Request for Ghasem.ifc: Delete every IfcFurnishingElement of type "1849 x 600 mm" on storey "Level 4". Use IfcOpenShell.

First a look at what the model holds.

```python
import ifcopenshell
import ifcopenshell.util.element

model = ifcopenshell.open("Ghasem.ifc")
print(model.schema)
storey = next(s for s in model.by_type("IfcBuildingStorey") if s.Name == "Level 4")
furniture = [e for e in ifcopenshell.util.element.get_decomposition(storey) if e.is_a("IfcFurnishingElement")]
seen = {}
for e in furniture:
    element_type = ifcopenshell.util.element.get_type(e)
    name = element_type.Name if element_type not in (None, e) else None
    seen[name] = seen.get(name, 0) + 1
for name, count in sorted(seen.items(), key=str):
    print(count, "x", name)
```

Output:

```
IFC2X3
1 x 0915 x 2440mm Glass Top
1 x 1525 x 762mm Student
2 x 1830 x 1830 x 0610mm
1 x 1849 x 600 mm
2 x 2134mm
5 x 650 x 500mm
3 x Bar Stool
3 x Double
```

```python
import ifcopenshell
import ifcopenshell.api.root
import ifcopenshell.util.element

model = ifcopenshell.open("Ghasem.ifc")

storey = next(s for s in model.by_type("IfcBuildingStorey") if s.Name == "Level 4")
furniture = [e for e in ifcopenshell.util.element.get_decomposition(storey) if e.is_a("IfcFurnishingElement")]
targets = [e for e in furniture if (t := ifcopenshell.util.element.get_type(e)) not in (None, e) and t.Name == "1849 x 600 mm"]

for e in targets:
    ifcopenshell.api.root.remove_product(model, product=e)
print(len(targets), "removed")

model.write("Ghasem-out.ifc")
```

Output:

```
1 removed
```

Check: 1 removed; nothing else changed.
